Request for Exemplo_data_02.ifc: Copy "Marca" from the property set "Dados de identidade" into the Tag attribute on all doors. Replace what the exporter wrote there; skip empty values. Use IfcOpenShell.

First a look at what the model holds.

```python
import ifcopenshell
import ifcopenshell.util.element

model = ifcopenshell.open("Exemplo_data_02.ifc")
print(model.schema)
doors = model.by_type("IfcDoor")
print(len(doors), "doors")
for e in doors[:8]:
    source = ifcopenshell.util.element.get_pset(e, "Dados de identidade", "Marca")
    target = e.Tag
    print(e.id(), repr(source), repr(target), sep=" | ")
```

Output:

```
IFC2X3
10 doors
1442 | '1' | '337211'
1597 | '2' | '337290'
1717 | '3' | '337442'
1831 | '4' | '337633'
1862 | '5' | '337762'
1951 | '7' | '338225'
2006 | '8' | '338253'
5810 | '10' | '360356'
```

```python
import ifcopenshell
import ifcopenshell.util.element

model = ifcopenshell.open("Exemplo_data_02.ifc")

count = 0
for e in model.by_type("IfcDoor"):
    value = ifcopenshell.util.element.get_pset(e, "Dados de identidade", "Marca")
    current = e.Tag
    if not value or not value.strip() or current == value:
        continue
    e.Tag = value
    count += 1

print(count, "doors updated")

model.write("Exemplo_data_02_updated.ifc")
```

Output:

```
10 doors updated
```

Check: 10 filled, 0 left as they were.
